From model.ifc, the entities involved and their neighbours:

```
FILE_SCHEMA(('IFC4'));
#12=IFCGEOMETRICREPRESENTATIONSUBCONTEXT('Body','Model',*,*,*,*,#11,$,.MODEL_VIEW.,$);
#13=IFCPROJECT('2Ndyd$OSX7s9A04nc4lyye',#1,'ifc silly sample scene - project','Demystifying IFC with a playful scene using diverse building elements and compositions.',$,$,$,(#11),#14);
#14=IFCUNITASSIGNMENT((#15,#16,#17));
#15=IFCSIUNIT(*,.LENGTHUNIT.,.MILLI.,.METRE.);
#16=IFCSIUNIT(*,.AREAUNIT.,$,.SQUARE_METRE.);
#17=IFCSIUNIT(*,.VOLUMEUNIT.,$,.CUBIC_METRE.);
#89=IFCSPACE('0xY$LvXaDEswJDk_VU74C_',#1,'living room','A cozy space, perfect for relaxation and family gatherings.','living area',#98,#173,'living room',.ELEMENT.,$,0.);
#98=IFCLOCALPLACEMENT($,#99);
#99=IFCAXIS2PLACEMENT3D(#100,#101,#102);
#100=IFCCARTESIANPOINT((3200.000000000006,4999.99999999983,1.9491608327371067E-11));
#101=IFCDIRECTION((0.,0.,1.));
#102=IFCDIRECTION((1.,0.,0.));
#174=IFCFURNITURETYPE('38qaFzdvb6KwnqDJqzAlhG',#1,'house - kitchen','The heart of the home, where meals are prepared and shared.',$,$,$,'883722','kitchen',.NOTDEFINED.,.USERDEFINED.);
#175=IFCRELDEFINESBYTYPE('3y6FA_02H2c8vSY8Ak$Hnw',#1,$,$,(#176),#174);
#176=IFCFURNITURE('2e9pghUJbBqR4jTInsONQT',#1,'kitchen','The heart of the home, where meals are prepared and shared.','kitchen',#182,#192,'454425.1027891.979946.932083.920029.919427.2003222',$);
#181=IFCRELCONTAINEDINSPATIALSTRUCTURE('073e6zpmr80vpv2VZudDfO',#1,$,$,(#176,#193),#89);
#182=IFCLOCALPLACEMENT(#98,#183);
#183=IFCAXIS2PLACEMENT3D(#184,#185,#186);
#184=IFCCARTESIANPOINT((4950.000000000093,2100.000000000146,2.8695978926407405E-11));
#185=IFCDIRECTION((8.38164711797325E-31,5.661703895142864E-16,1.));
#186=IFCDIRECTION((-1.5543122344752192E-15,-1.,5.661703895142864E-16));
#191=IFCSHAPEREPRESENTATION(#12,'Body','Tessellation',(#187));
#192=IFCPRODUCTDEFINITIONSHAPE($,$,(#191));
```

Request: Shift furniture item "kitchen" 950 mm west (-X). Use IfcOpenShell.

```python
import ifcopenshell
import ifcopenshell.api.geometry
import ifcopenshell.util.placement
import ifcopenshell.util.unit

model = ifcopenshell.open("model.ifc")
unit_scale = ifcopenshell.util.unit.calculate_unit_scale(model)

item = model.by_guid("2e9pghUJbBqR4jTInsONQT")
matrix = ifcopenshell.util.placement.get_local_placement(item.ObjectPlacement)
matrix[0, 3] -= 0.95 / unit_scale
ifcopenshell.api.geometry.edit_object_placement(model, product=item, matrix=matrix, is_si=False)

print(ifcopenshell.util.placement.get_local_placement(item.ObjectPlacement).round(3) + 0.0)

model.write("model_v2.ifc")
```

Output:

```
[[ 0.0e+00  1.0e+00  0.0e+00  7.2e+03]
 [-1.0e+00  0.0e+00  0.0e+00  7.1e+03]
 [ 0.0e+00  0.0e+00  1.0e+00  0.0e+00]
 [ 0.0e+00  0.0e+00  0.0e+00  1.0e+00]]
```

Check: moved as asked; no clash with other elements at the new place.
